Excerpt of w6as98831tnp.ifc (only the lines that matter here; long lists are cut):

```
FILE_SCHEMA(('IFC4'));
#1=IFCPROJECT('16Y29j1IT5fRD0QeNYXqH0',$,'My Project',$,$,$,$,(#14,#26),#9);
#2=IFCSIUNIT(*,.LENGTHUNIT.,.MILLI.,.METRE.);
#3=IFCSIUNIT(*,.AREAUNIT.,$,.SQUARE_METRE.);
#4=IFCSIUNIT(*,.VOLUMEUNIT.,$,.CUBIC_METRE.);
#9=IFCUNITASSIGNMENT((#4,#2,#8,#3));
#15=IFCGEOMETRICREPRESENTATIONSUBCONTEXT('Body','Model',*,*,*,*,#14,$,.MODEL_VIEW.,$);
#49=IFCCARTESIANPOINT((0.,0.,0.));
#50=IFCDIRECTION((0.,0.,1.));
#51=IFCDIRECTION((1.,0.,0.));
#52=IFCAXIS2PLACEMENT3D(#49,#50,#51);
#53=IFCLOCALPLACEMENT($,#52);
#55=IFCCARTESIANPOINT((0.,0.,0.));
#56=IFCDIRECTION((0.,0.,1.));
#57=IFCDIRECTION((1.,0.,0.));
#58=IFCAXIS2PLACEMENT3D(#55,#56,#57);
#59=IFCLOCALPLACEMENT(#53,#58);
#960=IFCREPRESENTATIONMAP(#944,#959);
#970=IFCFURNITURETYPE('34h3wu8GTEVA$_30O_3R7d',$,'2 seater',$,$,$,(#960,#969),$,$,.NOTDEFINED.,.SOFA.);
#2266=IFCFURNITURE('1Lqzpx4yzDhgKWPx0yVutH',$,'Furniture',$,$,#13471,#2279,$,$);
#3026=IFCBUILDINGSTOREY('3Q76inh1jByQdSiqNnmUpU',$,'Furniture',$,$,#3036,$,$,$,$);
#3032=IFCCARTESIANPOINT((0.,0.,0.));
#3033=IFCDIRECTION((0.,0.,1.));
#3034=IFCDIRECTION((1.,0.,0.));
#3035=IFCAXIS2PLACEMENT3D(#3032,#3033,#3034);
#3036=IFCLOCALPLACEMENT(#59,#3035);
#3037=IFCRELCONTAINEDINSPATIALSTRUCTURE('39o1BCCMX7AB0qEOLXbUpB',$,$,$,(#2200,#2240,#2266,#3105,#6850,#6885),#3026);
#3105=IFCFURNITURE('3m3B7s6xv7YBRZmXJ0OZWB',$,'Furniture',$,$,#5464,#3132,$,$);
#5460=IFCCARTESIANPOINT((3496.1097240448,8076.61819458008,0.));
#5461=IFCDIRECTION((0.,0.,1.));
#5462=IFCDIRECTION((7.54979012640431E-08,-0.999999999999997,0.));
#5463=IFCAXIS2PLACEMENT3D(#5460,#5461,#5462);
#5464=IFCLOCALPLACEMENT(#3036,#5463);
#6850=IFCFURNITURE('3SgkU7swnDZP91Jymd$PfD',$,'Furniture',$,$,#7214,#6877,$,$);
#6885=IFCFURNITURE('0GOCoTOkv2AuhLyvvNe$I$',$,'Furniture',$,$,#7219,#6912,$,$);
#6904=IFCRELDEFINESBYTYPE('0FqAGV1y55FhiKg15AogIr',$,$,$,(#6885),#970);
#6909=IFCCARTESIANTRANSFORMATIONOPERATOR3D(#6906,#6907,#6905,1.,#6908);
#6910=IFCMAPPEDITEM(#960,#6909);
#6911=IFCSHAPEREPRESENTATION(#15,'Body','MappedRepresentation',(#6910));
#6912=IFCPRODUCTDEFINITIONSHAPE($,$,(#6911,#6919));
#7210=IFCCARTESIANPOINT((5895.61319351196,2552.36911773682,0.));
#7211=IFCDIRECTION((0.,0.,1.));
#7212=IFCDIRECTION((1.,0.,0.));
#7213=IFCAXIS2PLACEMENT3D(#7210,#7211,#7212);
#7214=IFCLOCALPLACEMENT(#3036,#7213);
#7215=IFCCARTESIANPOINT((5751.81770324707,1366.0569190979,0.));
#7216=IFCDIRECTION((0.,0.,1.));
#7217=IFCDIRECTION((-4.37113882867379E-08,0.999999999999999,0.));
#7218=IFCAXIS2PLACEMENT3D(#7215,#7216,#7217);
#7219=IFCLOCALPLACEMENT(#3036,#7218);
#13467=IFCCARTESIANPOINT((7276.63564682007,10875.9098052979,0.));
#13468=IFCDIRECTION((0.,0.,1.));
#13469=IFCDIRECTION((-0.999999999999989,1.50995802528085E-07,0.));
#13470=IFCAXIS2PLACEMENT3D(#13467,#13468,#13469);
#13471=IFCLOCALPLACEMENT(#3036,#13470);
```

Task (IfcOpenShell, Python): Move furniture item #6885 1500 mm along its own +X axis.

```python
import ifcopenshell
import ifcopenshell.api.geometry
import ifcopenshell.util.placement

model = ifcopenshell.open("w6as98831tnp.ifc")

item = model.by_guid("0GOCoTOkv2AuhLyvvNe$I$")
matrix = ifcopenshell.util.placement.get_local_placement(item.ObjectPlacement)
matrix[:3, 3] += matrix[:3, 0] * 1500.0
ifcopenshell.api.geometry.edit_object_placement(model, product=item, matrix=matrix, is_si=False)

print(ifcopenshell.util.placement.get_local_placement(item.ObjectPlacement).round(3) + 0.0)

model.write("w6as98831tnp_v2.ifc")
```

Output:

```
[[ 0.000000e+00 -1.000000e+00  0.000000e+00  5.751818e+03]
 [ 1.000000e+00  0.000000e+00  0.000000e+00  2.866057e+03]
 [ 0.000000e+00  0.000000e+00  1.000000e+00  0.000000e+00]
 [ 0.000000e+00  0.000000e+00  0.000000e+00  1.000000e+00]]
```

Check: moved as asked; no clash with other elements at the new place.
